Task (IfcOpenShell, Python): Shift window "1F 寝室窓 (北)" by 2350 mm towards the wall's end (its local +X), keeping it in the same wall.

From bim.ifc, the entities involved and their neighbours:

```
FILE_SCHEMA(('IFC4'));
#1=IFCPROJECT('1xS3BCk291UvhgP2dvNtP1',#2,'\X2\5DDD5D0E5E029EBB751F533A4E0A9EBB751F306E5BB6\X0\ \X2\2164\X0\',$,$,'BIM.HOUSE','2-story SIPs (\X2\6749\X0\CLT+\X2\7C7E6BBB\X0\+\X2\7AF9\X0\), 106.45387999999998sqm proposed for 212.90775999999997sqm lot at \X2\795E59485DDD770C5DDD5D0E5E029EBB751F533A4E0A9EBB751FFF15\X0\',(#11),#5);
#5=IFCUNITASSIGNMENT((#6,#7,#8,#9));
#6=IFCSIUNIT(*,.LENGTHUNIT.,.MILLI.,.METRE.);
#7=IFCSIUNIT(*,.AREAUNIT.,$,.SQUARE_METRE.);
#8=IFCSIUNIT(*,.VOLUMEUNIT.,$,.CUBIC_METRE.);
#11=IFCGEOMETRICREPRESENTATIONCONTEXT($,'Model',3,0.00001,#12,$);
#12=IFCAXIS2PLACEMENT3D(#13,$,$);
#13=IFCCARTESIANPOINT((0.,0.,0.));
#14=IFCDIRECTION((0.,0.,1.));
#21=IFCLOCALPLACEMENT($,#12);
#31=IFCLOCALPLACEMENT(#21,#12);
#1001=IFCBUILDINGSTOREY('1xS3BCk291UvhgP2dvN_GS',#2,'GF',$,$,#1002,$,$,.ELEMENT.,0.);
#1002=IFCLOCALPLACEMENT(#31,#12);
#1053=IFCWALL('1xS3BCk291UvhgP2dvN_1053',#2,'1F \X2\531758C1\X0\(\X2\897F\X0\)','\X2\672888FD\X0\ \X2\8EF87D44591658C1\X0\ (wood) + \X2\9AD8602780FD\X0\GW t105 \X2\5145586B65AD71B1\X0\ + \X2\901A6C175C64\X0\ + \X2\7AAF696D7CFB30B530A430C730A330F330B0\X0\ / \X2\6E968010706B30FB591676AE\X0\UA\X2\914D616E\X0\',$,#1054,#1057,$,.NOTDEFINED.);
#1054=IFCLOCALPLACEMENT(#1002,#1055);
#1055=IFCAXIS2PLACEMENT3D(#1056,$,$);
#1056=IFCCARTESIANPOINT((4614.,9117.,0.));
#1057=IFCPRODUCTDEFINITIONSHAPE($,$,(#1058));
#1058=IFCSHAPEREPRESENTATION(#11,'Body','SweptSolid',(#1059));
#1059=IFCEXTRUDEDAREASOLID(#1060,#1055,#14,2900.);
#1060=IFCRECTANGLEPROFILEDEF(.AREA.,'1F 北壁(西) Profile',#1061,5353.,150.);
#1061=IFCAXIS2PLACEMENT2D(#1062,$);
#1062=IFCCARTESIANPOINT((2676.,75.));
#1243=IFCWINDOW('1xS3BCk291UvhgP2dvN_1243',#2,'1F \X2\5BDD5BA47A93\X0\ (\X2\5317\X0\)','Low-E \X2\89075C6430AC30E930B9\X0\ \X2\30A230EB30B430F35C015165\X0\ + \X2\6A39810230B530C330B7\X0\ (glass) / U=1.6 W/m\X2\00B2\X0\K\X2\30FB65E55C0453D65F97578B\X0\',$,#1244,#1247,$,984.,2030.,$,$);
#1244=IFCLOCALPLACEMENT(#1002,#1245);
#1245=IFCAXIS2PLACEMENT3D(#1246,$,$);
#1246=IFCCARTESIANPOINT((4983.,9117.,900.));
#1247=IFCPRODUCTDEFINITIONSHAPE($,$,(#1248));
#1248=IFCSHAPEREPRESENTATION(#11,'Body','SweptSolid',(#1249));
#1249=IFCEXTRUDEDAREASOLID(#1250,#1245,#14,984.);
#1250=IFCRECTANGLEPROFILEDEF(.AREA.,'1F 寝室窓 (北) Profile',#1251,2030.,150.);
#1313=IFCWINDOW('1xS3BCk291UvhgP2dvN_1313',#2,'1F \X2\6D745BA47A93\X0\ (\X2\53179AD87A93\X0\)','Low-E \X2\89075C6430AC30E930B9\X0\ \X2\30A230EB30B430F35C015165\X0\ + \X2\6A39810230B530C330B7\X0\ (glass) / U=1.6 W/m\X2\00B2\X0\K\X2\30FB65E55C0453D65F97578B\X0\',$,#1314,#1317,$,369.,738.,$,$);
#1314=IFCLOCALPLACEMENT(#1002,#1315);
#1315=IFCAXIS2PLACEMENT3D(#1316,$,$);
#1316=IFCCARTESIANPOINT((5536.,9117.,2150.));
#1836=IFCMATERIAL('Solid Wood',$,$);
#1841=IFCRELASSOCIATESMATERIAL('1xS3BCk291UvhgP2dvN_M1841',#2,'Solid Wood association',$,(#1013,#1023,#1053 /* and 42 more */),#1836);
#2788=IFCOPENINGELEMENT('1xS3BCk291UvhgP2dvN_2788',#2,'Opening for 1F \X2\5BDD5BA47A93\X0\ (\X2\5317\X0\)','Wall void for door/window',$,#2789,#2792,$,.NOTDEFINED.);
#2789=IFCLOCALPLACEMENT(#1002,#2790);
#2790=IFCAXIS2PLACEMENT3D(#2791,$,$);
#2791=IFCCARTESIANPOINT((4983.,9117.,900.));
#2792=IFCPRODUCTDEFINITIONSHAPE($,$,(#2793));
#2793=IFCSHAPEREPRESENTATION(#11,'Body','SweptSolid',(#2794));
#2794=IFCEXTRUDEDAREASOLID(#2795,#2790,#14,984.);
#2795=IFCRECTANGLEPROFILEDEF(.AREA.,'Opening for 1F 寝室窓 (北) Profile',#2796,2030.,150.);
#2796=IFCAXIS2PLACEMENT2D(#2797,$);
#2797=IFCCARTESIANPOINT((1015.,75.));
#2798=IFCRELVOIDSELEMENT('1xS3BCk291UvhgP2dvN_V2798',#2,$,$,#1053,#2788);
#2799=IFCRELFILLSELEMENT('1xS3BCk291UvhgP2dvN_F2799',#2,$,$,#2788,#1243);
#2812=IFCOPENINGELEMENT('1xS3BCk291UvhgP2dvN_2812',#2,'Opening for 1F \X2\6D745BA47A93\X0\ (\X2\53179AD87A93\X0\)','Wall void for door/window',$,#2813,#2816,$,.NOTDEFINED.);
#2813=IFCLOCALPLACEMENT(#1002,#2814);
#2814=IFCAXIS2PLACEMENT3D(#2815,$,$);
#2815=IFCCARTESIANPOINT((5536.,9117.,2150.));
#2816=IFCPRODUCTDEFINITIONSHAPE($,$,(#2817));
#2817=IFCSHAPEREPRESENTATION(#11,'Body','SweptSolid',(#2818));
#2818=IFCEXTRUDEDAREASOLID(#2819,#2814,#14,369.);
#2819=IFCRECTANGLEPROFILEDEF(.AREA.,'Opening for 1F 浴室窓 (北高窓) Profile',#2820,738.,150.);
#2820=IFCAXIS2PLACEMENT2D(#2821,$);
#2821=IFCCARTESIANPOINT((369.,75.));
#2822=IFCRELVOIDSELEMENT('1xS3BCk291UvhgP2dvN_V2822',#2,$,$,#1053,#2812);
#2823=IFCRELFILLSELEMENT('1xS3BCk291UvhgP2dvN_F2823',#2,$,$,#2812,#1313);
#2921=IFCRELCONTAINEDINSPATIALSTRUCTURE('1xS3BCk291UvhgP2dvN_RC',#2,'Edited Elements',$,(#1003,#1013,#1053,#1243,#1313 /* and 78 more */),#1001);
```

```python
import ifcopenshell
import ifcopenshell.api.geometry
import ifcopenshell.util.placement
import ifcopenshell.util.unit

model = ifcopenshell.open("bim.ifc")
unit_scale = ifcopenshell.util.unit.calculate_unit_scale(model)

window = model.by_guid("1xS3BCk291UvhgP2dvN_1243")
opening = window.FillsVoids[0].RelatingOpeningElement
wall = opening.VoidsElements[0].RelatingBuildingElement

wall_matrix = ifcopenshell.util.placement.get_local_placement(wall.ObjectPlacement)
shift = wall_matrix[:3, 0] * 2.35 / unit_scale
before = ifcopenshell.util.placement.get_local_placement(window.ObjectPlacement)[:3, 3].copy()

# The window is not placed relative to its opening, so move both.
for product in (opening, window):
    matrix = ifcopenshell.util.placement.get_local_placement(product.ObjectPlacement)
    matrix[:3, 3] += shift
    ifcopenshell.api.geometry.edit_object_placement(model, product=product, matrix=matrix, is_si=False)

after = ifcopenshell.util.placement.get_local_placement(window.ObjectPlacement)[:3, 3]
print("window moved by", (after - before).round(3) + 0.0)

model.write("bim_rev.ifc")
```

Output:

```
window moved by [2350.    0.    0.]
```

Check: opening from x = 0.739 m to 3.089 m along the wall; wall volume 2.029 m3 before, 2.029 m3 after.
